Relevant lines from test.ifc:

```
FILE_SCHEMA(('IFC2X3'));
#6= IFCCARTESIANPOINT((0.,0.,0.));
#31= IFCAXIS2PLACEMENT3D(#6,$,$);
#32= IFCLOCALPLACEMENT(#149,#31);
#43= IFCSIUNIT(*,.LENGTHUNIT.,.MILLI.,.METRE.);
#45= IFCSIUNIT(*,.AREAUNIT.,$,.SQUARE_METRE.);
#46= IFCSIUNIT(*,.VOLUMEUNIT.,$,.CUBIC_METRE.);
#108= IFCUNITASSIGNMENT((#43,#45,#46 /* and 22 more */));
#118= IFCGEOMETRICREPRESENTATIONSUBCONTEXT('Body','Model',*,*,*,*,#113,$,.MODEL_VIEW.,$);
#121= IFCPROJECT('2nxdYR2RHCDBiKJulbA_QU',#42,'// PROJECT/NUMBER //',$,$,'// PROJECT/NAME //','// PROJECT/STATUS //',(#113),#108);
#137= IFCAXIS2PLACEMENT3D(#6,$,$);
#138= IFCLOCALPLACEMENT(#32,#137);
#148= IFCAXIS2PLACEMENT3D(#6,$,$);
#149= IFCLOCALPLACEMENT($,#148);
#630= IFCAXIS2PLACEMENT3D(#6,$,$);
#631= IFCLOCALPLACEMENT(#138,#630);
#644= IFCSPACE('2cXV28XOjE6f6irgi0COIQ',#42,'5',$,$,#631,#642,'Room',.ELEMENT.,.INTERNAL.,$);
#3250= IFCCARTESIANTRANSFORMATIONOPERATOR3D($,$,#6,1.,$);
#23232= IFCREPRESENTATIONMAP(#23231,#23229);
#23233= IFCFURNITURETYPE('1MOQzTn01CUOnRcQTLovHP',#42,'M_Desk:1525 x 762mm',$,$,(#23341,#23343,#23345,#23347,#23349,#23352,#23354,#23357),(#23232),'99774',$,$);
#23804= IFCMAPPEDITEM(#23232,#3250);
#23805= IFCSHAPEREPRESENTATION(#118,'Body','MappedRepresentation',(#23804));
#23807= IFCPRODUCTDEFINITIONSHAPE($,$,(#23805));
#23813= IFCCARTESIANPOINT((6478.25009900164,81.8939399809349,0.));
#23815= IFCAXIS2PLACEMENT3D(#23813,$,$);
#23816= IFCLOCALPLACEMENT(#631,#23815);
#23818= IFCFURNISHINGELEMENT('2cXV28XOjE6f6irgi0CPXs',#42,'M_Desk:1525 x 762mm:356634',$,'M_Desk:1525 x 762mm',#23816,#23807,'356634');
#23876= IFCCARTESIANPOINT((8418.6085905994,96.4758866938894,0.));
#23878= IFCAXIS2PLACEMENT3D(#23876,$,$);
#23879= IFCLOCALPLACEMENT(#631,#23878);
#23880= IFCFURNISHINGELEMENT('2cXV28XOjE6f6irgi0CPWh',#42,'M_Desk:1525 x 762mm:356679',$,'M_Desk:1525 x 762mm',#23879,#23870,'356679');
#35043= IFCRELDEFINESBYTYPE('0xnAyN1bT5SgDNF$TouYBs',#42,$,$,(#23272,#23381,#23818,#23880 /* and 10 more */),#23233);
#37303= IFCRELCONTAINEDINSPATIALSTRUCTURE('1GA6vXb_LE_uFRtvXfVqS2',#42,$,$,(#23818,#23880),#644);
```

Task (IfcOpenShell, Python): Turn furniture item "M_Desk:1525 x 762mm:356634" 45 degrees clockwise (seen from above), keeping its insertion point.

```python
import ifcopenshell
import ifcopenshell.api.geometry
import ifcopenshell.util.placement

model = ifcopenshell.open("test.ifc")

item = model.by_guid("2cXV28XOjE6f6irgi0CPXs")
matrix = ifcopenshell.util.placement.get_local_placement(item.ObjectPlacement)
matrix = matrix @ ifcopenshell.util.placement.rotation(-45, "Z")
ifcopenshell.api.geometry.edit_object_placement(model, product=item, matrix=matrix, is_si=False)

print(ifcopenshell.util.placement.get_local_placement(item.ObjectPlacement).round(3) + 0.0)

model.write("test_updated.ifc")
```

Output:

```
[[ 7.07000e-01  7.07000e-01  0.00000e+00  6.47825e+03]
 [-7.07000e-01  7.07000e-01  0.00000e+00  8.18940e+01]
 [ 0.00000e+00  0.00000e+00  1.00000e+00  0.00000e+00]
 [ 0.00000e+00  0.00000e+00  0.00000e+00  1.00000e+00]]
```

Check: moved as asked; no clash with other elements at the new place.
